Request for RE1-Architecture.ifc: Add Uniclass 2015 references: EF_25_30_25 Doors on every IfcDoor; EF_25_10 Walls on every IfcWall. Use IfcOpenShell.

First a look at what the model holds.

```python
import ifcopenshell

model = ifcopenshell.open("RE1-Architecture.ifc")
print(model.schema)
print("classifications:", [c.Name for c in model.by_type("IfcClassification")])
for ifc_class in ("IfcDoor", "IfcRoof", "IfcStair", "IfcWall", "IfcWindow"):
    print(ifc_class, len(model.by_type(ifc_class)))
```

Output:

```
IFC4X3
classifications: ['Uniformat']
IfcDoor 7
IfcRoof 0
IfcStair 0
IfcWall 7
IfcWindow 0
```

```python
import ifcopenshell
import ifcopenshell.api.classification

model = ifcopenshell.open("RE1-Architecture.ifc")

system = ifcopenshell.api.classification.add_classification(model, classification="Uniclass 2015")

codes = {
    "IfcDoor": ("EF_25_30_25", "Doors"),
    "IfcWall": ("EF_25_10", "Walls"),
}
for ifc_class, (code, name) in codes.items():
    products = model.by_type(ifc_class)
    ifcopenshell.api.classification.add_reference(
        model, products=products, classification=system, identification=code, name=name
    )
    print(code, len(products))

model.write("RE1-Architecture_updated.ifc")
```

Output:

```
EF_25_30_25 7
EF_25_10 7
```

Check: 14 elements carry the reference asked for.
